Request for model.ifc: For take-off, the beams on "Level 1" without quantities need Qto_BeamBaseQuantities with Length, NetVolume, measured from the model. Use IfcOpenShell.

First a look at what the model holds.

```python
import ifcopenshell
import ifcopenshell.util.element
import ifcopenshell.util.unit

model = ifcopenshell.open("model.ifc")
print(model.schema)
for unit_type in ("LENGTHUNIT", "AREAUNIT", "VOLUMEUNIT"):
    print(unit_type, ifcopenshell.util.unit.calculate_unit_scale(model, unit_type))
storey = next(s for s in model.by_type("IfcBuildingStorey") if s.Name == "Level 1")
beams = [e for e in ifcopenshell.util.element.get_decomposition(storey) if e.is_a("IfcBeam")]
for e in sorted(beams, key=lambda e: e.id()):
    print(e.id(), e.is_a(), e.Name, list(ifcopenshell.util.element.get_psets(e, qtos_only=True)), sep=" | ")
```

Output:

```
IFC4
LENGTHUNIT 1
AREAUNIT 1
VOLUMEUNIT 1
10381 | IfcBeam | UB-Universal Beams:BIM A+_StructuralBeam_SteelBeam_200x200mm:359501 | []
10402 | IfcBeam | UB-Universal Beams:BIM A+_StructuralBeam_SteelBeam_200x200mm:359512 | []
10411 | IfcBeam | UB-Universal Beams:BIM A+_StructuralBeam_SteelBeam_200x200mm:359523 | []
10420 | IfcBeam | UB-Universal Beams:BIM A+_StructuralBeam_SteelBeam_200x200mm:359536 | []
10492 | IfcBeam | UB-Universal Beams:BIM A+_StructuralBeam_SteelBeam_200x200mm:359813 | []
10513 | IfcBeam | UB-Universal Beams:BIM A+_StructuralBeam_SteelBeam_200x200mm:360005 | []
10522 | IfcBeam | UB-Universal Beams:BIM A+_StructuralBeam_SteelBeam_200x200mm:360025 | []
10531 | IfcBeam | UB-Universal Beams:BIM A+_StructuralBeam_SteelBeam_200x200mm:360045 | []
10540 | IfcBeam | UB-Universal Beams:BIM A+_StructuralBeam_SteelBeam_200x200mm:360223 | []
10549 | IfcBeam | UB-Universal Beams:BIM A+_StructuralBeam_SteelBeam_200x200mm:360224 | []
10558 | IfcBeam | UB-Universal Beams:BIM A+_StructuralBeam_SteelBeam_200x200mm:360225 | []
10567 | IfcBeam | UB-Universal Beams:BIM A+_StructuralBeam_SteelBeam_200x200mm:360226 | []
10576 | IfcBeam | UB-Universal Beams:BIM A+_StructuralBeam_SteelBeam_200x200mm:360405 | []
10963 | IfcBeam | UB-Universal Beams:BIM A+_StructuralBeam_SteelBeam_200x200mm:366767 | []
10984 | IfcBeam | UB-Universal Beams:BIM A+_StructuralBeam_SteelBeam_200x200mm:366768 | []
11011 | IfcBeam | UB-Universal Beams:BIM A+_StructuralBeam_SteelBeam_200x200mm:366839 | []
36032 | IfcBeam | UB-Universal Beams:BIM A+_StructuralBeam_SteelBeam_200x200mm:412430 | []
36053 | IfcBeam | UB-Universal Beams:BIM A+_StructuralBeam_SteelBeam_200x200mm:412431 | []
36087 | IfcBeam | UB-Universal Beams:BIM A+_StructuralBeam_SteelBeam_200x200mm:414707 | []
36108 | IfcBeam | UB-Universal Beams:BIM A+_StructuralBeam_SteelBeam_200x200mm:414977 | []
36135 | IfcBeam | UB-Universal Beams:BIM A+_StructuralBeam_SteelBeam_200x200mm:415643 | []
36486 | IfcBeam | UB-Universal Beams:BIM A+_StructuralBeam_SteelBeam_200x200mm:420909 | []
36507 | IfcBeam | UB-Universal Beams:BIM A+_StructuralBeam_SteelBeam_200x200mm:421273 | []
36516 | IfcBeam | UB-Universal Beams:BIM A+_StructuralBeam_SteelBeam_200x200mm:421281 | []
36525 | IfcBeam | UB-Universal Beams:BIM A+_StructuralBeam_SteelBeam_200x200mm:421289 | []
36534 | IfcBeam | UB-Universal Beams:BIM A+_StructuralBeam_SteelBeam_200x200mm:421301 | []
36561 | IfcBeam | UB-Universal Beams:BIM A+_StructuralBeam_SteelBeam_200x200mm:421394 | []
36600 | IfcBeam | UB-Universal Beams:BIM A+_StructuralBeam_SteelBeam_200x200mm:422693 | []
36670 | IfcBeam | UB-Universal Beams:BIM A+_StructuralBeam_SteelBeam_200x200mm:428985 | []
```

```python
import ifcopenshell
import ifcopenshell.api.pset
import ifcopenshell.geom
import ifcopenshell.util.element
import ifcopenshell.util.shape
import ifcopenshell.util.unit

model = ifcopenshell.open("model.ifc")
unit_scale = ifcopenshell.util.unit.calculate_unit_scale(model)
volume_scale = ifcopenshell.util.unit.calculate_unit_scale(model, "VOLUMEUNIT")
settings = ifcopenshell.geom.settings()

storey = next(s for s in model.by_type("IfcBuildingStorey") if s.Name == "Level 1")
beams = [e for e in ifcopenshell.util.element.get_decomposition(storey) if e.is_a("IfcBeam")]

for e in sorted(beams, key=lambda e: e.id()):
    if ifcopenshell.util.element.get_psets(e, qtos_only=True, should_inherit=False):
        continue
    # Geometry comes back in metres, in the element's own axes.
    shape = ifcopenshell.geom.create_shape(settings, e)
    values = {
        "Length": ifcopenshell.util.shape.get_max_xyz(shape.geometry) / unit_scale,
        "NetVolume": ifcopenshell.util.shape.get_volume(shape.geometry) / volume_scale,
    }
    qto = ifcopenshell.api.pset.add_qto(model, product=e, name="Qto_BeamBaseQuantities")
    ifcopenshell.api.pset.edit_qto(model, qto=qto, properties=values)
    print(e.id(), {k: round(v, 3) for k, v in values.items()})

model.write("model_v2.ifc")
```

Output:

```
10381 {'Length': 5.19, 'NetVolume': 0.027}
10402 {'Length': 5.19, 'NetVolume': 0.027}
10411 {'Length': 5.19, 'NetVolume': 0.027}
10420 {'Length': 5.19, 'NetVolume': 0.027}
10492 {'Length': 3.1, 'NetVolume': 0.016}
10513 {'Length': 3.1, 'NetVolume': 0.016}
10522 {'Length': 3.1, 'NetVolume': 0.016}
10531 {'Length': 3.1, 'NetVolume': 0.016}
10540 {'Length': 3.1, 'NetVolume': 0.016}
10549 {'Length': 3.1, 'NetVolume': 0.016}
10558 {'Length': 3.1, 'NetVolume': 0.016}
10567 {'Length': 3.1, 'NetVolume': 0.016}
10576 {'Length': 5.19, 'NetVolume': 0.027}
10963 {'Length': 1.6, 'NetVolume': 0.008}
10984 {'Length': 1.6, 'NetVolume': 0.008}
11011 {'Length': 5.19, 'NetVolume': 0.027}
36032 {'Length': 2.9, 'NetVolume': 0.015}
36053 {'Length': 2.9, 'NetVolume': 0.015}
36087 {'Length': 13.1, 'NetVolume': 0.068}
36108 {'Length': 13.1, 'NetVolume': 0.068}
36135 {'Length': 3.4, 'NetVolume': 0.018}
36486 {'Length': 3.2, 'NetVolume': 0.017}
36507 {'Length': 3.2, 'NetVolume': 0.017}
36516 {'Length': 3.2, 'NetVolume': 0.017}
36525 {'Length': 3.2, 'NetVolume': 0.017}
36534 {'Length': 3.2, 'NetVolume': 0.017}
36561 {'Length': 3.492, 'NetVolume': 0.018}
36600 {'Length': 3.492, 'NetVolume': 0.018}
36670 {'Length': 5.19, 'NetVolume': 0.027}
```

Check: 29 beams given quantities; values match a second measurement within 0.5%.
